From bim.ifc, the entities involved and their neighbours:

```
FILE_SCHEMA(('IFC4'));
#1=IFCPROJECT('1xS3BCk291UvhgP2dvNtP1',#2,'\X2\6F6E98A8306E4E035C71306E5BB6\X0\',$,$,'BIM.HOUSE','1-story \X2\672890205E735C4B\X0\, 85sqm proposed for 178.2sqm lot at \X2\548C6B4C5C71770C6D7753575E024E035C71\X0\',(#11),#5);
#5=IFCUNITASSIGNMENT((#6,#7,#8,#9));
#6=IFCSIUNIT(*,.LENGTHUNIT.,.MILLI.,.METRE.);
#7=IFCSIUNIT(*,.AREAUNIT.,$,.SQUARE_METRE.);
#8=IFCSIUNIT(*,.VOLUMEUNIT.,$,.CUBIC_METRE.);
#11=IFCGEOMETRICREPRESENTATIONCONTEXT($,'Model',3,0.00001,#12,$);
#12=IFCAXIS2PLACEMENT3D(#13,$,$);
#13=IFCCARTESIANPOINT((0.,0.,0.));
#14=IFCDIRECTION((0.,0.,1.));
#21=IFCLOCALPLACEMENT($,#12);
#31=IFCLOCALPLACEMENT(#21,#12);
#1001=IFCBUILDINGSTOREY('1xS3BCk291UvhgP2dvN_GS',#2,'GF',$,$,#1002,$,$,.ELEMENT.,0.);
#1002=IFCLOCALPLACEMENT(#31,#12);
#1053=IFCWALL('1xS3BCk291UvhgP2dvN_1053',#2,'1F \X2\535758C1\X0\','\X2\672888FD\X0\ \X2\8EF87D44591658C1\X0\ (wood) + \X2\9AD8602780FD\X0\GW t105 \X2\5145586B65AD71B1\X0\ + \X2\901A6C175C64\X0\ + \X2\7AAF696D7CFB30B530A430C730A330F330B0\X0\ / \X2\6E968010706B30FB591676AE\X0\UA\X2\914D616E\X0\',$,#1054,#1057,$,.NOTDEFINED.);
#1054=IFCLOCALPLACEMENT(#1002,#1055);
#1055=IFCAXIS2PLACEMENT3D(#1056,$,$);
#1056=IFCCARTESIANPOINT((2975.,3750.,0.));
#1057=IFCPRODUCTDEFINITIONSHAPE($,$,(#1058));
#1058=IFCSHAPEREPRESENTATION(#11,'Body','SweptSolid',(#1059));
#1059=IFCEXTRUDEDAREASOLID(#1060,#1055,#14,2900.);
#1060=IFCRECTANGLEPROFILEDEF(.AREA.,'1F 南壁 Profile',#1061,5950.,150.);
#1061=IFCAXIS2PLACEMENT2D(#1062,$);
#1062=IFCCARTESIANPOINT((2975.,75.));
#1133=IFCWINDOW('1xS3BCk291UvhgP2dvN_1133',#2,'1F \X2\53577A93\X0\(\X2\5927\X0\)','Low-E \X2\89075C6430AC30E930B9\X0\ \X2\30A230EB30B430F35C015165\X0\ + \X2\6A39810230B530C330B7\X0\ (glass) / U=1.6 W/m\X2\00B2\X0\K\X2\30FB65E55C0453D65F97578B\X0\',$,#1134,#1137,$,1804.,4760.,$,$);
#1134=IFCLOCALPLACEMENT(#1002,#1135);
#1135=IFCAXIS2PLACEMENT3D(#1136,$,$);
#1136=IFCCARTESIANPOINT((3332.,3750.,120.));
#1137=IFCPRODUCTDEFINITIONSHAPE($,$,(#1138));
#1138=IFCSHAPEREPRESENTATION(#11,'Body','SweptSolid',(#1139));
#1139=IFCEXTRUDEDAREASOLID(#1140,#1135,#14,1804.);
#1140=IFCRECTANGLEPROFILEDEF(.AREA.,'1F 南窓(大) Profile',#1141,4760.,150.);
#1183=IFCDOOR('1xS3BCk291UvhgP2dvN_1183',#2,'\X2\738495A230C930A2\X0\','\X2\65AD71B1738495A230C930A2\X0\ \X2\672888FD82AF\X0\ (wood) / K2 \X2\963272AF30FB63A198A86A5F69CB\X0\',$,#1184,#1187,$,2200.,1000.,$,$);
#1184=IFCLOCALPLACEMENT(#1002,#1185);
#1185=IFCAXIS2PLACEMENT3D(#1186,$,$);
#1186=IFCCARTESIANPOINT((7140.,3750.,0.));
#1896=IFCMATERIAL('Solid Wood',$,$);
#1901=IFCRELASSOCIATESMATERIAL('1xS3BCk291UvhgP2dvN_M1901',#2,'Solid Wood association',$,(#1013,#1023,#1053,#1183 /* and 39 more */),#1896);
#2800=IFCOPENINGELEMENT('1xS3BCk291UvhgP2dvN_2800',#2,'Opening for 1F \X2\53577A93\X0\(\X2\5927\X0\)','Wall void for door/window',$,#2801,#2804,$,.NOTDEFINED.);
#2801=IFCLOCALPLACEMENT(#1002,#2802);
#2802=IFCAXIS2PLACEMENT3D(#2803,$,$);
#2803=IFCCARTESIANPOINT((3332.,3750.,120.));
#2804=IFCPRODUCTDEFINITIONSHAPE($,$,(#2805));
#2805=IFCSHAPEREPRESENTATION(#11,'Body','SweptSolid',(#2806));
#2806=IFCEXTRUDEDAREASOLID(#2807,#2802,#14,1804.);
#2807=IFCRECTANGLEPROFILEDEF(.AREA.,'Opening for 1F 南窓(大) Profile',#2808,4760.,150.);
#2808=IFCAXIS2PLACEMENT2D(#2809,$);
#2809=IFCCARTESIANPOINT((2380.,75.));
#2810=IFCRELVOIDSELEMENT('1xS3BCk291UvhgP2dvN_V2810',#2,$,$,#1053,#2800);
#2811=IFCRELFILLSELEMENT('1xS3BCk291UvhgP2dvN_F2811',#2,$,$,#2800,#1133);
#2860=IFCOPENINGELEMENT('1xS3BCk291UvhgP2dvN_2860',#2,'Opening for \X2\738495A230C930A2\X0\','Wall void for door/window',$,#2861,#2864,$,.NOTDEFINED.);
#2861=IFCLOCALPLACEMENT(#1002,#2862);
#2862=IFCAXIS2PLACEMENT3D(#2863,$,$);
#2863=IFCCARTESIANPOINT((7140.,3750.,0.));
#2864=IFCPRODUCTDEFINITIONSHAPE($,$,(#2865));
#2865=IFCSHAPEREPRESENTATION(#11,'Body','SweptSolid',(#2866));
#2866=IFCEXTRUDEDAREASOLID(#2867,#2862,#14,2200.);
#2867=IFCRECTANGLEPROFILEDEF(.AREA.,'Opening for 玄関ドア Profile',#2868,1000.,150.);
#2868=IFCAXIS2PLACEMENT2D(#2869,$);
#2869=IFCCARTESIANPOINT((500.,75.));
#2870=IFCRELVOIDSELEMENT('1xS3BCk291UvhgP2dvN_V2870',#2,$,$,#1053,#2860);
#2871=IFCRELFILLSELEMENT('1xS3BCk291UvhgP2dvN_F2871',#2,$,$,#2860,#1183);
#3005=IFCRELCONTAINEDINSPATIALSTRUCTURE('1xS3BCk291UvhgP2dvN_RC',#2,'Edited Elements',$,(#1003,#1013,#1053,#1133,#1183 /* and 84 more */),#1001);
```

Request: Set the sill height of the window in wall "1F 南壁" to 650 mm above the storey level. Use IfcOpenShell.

```python
import numpy as np
import ifcopenshell
import ifcopenshell.api.geometry
import ifcopenshell.geom
import ifcopenshell.util.element
import ifcopenshell.util.placement
import ifcopenshell.util.shape
import ifcopenshell.util.unit

model = ifcopenshell.open("bim.ifc")
unit_scale = ifcopenshell.util.unit.calculate_unit_scale(model)

window = model.by_id(1133)
opening = window.FillsVoids[0].RelatingOpeningElement
storey = ifcopenshell.util.element.get_container(window, ifc_class="IfcBuildingStorey")
level = ifcopenshell.util.placement.get_local_placement(storey.ObjectPlacement)[2, 3]

# The opening's origin need not be at the sill, so measure its lowest point.
shape = ifcopenshell.geom.create_shape(ifcopenshell.geom.settings(), opening)
bottom = ifcopenshell.util.shape.get_shape_bottom_elevation(shape, shape.geometry) / unit_scale
dz = level + 0.65 / unit_scale - bottom

shift = np.array([0.0, 0.0, dz])
# The window is not placed relative to its opening, so move both.
for product in (opening, window):
    matrix = ifcopenshell.util.placement.get_local_placement(product.ObjectPlacement)
    matrix[:3, 3] += shift
    ifcopenshell.api.geometry.edit_object_placement(model, product=product, matrix=matrix, is_si=False)

print(f"moved by {dz * unit_scale:+.3f} m")

model.write("bim-out.ifc")
```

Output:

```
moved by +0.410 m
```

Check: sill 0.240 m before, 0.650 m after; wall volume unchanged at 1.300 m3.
